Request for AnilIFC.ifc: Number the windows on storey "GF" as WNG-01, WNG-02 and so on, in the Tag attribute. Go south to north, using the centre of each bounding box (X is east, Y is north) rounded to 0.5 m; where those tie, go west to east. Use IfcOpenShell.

First a look at what the model holds.

```python
import ifcopenshell
import ifcopenshell.util.element
import ifcopenshell.util.placement

model = ifcopenshell.open("AnilIFC.ifc")
print(model.schema)
storey = next(s for s in model.by_type("IfcBuildingStorey") if s.Name == "GF")
windows = [e for e in ifcopenshell.util.element.get_decomposition(storey) if e.is_a("IfcWindow")]
for e in sorted(windows, key=lambda e: e.id()):
    origin = ifcopenshell.util.placement.get_local_placement(e.ObjectPlacement)[:3, 3]
    print(e.id(), e.Tag, e.Name, origin.round(2) + 0.0, sep=" | ")
```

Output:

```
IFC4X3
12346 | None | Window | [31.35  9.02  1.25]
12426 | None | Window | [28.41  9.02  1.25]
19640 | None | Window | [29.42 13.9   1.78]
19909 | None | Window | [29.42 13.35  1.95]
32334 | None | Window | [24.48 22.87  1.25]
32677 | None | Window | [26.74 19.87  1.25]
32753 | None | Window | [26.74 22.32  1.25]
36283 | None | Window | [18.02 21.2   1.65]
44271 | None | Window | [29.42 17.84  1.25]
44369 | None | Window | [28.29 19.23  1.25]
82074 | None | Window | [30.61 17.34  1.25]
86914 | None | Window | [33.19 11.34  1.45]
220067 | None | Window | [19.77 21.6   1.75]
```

```python
import ifcopenshell
import ifcopenshell.geom
import ifcopenshell.util.element
import ifcopenshell.util.shape

model = ifcopenshell.open("AnilIFC.ifc")
settings = ifcopenshell.geom.settings()
settings.set("use-world-coords", True)


def centre(element):
    shape = ifcopenshell.geom.create_shape(settings, element)
    return ifcopenshell.util.shape.get_bbox_centroid(shape.geometry)


storey = next(s for s in model.by_type("IfcBuildingStorey") if s.Name == "GF")
windows = [e for e in ifcopenshell.util.element.get_decomposition(storey) if e.is_a("IfcWindow")]

# Insertion points can sit at a corner or the storey origin, so sort by the geometry (in metres).
centres = {e: centre(e) for e in windows}
windows.sort(key=lambda e: (round(centres[e][1] / 0.5), centres[e][0]))

for i, e in enumerate(windows, start=1):
    number = f"WNG-{i:02d}"
    e.Tag = number
    print(e.id(), number)

model.write("AnilIFC-out.ifc")
```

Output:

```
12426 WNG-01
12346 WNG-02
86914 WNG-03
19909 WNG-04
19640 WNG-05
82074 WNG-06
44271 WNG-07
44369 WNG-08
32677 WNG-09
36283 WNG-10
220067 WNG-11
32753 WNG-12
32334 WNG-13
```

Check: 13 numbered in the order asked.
